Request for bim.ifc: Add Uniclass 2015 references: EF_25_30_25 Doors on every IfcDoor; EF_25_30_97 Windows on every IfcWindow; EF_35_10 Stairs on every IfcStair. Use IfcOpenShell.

First a look at what the model holds.

```python
import ifcopenshell

model = ifcopenshell.open("bim.ifc")
print(model.schema)
print("classifications:", [c.Name for c in model.by_type("IfcClassification")])
for ifc_class in ("IfcDoor", "IfcRoof", "IfcStair", "IfcWall", "IfcWindow"):
    print(ifc_class, len(model.by_type(ifc_class)))
```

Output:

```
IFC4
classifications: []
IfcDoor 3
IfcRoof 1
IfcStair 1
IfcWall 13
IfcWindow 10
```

```python
import ifcopenshell
import ifcopenshell.api.classification

model = ifcopenshell.open("bim.ifc")

system = ifcopenshell.api.classification.add_classification(model, classification="Uniclass 2015")

codes = {
    "IfcDoor": ("EF_25_30_25", "Doors"),
    "IfcWindow": ("EF_25_30_97", "Windows"),
    "IfcStair": ("EF_35_10", "Stairs"),
}
for ifc_class, (code, name) in codes.items():
    products = model.by_type(ifc_class)
    ifcopenshell.api.classification.add_reference(
        model, products=products, classification=system, identification=code, name=name
    )
    print(code, len(products))

model.write("bim_v2.ifc")
```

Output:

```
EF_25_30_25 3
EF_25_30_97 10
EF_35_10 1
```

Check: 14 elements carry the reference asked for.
